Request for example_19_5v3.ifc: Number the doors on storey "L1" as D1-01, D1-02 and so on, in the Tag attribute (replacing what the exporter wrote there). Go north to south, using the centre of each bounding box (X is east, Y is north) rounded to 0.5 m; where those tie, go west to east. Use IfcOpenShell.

First a look at what the model holds.

```python
import ifcopenshell
import ifcopenshell.util.element
import ifcopenshell.util.placement

model = ifcopenshell.open("example_19_5v3.ifc")
print(model.schema)
storey = next(s for s in model.by_type("IfcBuildingStorey") if s.Name == "L1")
doors = [e for e in ifcopenshell.util.element.get_decomposition(storey) if e.is_a("IfcDoor")]
for e in sorted(doors, key=lambda e: e.id()):
    origin = ifcopenshell.util.placement.get_local_placement(e.ObjectPlacement)[:3, 3]
    print(e.id(), e.Tag, e.Name, origin.round(2) + 0.0, sep=" | ")
```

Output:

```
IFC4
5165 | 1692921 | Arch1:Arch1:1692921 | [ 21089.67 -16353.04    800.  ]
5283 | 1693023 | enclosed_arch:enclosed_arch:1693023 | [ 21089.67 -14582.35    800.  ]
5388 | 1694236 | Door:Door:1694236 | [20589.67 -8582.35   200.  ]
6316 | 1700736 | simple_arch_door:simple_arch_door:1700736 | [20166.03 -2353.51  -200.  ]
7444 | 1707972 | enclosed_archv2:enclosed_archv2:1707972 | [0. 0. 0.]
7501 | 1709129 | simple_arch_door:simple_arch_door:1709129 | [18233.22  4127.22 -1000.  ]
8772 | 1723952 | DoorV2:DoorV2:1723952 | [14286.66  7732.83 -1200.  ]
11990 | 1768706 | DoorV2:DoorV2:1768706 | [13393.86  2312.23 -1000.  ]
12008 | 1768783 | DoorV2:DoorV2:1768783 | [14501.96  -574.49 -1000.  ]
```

```python
import ifcopenshell
import ifcopenshell.geom
import ifcopenshell.util.element
import ifcopenshell.util.shape

model = ifcopenshell.open("example_19_5v3.ifc")
settings = ifcopenshell.geom.settings()
settings.set("use-world-coords", True)


def centre(element):
    shape = ifcopenshell.geom.create_shape(settings, element)
    return ifcopenshell.util.shape.get_bbox_centroid(shape.geometry)


storey = next(s for s in model.by_type("IfcBuildingStorey") if s.Name == "L1")
doors = [e for e in ifcopenshell.util.element.get_decomposition(storey) if e.is_a("IfcDoor")]

# Insertion points can sit at a corner or the storey origin, so sort by the geometry (in metres).
centres = {e: centre(e) for e in doors}
doors.sort(key=lambda e: (-round(centres[e][1] / 0.5), centres[e][0]))

for i, e in enumerate(doors, start=1):
    number = f"D1-{i:02d}"
    e.Tag = number
    print(e.id(), number)

model.write("example_19_5v3_updated.ifc")
```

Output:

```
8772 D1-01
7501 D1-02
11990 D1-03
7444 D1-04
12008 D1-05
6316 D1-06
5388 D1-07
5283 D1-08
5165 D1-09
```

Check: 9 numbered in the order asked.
